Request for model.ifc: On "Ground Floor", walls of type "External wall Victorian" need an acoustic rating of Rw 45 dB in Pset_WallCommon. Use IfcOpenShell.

First a look at what the model holds.

```python
import ifcopenshell
import ifcopenshell.util.element

model = ifcopenshell.open("model.ifc")
print(model.schema)
storey = next(s for s in model.by_type("IfcBuildingStorey") if s.Name == "Ground Floor")
walls = [e for e in ifcopenshell.util.element.get_decomposition(storey) if e.is_a("IfcWall")]
seen = {}
for e in walls:
    element_type = ifcopenshell.util.element.get_type(e)
    key = (element_type.Name if element_type != e and element_type else None, ifcopenshell.util.element.get_pset(e, "Pset_WallCommon", "AcousticRating"))
    seen[key] = seen.get(key, 0) + 1
for (name, value), count in sorted(seen.items(), key=str):
    print(count, "x", name, "|", value)
```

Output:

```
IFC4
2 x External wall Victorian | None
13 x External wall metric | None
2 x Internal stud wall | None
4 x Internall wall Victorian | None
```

```python
import ifcopenshell
import ifcopenshell.api.pset
import ifcopenshell.util.element

model = ifcopenshell.open("model.ifc")

storey = next(s for s in model.by_type("IfcBuildingStorey") if s.Name == "Ground Floor")
walls = [e for e in ifcopenshell.util.element.get_decomposition(storey) if e.is_a("IfcWall")]

count = 0
for e in walls:
    element_type = ifcopenshell.util.element.get_type(e)
    if element_type in (None, e) or element_type.Name != "External wall Victorian":
        continue
    # add_pset returns the element's existing set when there is one.
    pset = ifcopenshell.api.pset.add_pset(model, product=e, name="Pset_WallCommon")
    ifcopenshell.api.pset.edit_pset(model, pset=pset, properties={"AcousticRating": "Rw 45 dB"})
    count += 1

print(count, "walls updated")

model.write("model_v2.ifc")
```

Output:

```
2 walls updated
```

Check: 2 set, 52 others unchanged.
